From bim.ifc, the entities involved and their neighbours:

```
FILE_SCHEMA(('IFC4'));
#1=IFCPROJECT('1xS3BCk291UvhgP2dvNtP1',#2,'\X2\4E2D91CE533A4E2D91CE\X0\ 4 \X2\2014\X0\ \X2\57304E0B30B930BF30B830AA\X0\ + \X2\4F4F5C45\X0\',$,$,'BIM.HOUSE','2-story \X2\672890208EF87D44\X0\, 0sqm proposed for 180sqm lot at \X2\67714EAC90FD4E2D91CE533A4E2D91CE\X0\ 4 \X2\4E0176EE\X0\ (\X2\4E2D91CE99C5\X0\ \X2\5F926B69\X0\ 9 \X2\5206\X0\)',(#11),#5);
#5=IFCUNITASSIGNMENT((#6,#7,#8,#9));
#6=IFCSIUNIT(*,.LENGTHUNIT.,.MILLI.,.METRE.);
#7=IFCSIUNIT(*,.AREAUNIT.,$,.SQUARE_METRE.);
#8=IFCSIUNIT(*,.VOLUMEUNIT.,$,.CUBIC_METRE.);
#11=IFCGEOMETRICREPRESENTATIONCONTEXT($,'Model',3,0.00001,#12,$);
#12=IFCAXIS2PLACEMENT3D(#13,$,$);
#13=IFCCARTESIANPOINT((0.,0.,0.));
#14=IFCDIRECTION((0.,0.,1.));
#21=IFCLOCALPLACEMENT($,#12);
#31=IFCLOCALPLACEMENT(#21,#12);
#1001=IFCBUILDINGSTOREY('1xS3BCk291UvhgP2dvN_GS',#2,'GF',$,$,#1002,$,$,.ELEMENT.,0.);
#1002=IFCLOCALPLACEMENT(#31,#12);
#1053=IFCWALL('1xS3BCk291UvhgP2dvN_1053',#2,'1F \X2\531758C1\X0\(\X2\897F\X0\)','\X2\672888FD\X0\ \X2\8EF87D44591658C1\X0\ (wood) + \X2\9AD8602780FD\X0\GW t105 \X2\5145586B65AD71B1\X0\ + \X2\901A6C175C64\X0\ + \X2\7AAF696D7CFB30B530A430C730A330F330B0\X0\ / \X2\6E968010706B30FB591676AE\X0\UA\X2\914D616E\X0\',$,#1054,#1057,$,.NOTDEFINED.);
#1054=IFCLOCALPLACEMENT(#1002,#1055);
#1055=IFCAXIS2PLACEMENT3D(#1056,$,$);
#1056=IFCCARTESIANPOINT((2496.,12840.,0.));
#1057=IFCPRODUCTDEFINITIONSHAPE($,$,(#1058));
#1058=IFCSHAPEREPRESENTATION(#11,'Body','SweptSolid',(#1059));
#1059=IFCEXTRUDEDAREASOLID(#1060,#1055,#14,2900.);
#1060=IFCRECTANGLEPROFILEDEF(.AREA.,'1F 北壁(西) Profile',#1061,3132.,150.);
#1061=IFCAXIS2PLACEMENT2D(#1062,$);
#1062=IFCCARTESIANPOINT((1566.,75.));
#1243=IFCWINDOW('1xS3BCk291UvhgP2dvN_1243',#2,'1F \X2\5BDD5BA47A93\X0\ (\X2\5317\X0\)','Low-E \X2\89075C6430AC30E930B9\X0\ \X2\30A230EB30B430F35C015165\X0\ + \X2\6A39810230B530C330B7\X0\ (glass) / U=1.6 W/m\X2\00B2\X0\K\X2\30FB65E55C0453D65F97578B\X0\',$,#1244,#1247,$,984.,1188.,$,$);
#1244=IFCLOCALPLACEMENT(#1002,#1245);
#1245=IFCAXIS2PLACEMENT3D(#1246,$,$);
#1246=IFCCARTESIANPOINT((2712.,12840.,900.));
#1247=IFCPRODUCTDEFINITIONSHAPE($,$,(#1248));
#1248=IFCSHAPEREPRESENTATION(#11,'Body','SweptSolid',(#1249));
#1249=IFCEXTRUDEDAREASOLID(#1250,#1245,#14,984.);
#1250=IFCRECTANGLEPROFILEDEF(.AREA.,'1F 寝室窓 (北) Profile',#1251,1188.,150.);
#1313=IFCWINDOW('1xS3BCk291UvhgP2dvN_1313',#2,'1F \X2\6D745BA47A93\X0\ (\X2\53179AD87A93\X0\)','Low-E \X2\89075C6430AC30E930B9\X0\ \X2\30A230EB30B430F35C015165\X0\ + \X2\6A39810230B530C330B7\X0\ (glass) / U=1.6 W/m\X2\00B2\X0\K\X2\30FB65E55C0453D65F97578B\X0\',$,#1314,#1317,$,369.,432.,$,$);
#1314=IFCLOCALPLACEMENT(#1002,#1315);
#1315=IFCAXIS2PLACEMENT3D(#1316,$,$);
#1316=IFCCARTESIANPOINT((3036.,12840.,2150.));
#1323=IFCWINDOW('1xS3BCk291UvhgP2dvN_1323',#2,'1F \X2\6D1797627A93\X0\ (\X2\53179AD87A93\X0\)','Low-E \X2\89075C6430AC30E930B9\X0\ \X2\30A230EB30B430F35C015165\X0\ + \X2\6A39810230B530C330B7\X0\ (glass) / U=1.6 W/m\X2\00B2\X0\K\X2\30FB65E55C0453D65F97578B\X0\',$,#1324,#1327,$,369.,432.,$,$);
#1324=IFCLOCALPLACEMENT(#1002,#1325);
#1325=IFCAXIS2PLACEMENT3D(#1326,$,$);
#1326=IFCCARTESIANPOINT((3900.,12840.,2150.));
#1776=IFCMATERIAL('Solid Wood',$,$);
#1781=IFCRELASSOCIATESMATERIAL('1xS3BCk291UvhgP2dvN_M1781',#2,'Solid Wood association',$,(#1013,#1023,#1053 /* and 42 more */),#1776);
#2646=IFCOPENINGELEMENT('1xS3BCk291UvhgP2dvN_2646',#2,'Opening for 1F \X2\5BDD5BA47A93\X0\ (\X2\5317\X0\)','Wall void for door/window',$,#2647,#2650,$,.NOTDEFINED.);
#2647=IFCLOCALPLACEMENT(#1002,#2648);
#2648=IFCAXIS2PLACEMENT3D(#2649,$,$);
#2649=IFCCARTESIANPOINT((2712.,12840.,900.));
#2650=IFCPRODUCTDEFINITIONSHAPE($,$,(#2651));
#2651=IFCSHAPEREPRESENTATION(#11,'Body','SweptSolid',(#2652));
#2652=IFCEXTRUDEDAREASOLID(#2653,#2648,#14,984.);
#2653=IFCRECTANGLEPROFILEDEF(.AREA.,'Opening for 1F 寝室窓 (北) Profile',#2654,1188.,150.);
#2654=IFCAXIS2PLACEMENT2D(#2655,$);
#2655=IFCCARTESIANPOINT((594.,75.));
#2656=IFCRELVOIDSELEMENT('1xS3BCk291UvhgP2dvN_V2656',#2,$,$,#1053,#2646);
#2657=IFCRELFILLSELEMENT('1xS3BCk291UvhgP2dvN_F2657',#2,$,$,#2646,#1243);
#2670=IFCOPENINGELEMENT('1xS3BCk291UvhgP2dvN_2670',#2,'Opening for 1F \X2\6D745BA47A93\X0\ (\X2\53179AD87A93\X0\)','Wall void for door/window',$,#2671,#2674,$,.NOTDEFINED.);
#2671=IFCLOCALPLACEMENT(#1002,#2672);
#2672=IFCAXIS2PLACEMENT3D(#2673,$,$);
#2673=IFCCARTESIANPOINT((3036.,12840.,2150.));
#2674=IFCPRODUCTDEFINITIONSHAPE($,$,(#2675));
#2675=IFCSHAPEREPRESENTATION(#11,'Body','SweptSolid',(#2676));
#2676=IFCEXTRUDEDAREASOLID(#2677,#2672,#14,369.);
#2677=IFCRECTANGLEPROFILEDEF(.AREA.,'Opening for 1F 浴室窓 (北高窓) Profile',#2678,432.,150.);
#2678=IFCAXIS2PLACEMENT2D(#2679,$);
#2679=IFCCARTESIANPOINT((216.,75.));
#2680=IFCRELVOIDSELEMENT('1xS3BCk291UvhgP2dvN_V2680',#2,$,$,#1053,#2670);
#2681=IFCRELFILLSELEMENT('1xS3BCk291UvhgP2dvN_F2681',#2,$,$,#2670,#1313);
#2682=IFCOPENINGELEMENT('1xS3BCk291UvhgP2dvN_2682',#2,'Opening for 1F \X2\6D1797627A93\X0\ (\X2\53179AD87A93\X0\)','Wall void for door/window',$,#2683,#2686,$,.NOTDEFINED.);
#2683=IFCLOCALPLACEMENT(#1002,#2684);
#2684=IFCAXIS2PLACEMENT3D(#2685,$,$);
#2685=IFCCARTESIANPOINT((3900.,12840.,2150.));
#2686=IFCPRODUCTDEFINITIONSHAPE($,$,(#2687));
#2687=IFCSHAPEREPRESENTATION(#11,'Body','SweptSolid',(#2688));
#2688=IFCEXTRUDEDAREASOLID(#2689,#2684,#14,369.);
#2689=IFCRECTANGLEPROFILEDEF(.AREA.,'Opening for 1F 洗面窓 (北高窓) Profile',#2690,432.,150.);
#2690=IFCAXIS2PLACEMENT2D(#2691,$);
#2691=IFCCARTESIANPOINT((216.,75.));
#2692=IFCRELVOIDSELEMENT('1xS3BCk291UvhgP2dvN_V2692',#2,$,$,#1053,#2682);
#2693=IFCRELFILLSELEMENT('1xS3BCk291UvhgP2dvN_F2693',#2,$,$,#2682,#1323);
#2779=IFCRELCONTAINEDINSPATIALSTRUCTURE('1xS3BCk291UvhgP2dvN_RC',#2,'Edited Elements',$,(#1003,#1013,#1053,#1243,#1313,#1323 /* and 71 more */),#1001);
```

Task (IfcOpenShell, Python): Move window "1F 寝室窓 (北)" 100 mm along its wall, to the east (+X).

```python
import ifcopenshell
import ifcopenshell.api.geometry
import ifcopenshell.util.placement
import ifcopenshell.util.unit

model = ifcopenshell.open("bim.ifc")
unit_scale = ifcopenshell.util.unit.calculate_unit_scale(model)

window = model.by_guid("1xS3BCk291UvhgP2dvN_1243")
opening = window.FillsVoids[0].RelatingOpeningElement
wall = opening.VoidsElements[0].RelatingBuildingElement

wall_matrix = ifcopenshell.util.placement.get_local_placement(wall.ObjectPlacement)
shift = wall_matrix[:3, 0] * 0.1 / unit_scale
before = ifcopenshell.util.placement.get_local_placement(window.ObjectPlacement)[:3, 3].copy()

# The window is not placed relative to its opening, so move both.
for product in (opening, window):
    matrix = ifcopenshell.util.placement.get_local_placement(product.ObjectPlacement)
    matrix[:3, 3] += shift
    ifcopenshell.api.geometry.edit_object_placement(model, product=product, matrix=matrix, is_si=False)

after = ifcopenshell.util.placement.get_local_placement(window.ObjectPlacement)[:3, 3]
print("window moved by", (after - before).round(3) + 0.0)

model.write("bim_updated.ifc")
```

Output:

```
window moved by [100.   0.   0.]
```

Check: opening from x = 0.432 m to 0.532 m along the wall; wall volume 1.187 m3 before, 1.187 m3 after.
